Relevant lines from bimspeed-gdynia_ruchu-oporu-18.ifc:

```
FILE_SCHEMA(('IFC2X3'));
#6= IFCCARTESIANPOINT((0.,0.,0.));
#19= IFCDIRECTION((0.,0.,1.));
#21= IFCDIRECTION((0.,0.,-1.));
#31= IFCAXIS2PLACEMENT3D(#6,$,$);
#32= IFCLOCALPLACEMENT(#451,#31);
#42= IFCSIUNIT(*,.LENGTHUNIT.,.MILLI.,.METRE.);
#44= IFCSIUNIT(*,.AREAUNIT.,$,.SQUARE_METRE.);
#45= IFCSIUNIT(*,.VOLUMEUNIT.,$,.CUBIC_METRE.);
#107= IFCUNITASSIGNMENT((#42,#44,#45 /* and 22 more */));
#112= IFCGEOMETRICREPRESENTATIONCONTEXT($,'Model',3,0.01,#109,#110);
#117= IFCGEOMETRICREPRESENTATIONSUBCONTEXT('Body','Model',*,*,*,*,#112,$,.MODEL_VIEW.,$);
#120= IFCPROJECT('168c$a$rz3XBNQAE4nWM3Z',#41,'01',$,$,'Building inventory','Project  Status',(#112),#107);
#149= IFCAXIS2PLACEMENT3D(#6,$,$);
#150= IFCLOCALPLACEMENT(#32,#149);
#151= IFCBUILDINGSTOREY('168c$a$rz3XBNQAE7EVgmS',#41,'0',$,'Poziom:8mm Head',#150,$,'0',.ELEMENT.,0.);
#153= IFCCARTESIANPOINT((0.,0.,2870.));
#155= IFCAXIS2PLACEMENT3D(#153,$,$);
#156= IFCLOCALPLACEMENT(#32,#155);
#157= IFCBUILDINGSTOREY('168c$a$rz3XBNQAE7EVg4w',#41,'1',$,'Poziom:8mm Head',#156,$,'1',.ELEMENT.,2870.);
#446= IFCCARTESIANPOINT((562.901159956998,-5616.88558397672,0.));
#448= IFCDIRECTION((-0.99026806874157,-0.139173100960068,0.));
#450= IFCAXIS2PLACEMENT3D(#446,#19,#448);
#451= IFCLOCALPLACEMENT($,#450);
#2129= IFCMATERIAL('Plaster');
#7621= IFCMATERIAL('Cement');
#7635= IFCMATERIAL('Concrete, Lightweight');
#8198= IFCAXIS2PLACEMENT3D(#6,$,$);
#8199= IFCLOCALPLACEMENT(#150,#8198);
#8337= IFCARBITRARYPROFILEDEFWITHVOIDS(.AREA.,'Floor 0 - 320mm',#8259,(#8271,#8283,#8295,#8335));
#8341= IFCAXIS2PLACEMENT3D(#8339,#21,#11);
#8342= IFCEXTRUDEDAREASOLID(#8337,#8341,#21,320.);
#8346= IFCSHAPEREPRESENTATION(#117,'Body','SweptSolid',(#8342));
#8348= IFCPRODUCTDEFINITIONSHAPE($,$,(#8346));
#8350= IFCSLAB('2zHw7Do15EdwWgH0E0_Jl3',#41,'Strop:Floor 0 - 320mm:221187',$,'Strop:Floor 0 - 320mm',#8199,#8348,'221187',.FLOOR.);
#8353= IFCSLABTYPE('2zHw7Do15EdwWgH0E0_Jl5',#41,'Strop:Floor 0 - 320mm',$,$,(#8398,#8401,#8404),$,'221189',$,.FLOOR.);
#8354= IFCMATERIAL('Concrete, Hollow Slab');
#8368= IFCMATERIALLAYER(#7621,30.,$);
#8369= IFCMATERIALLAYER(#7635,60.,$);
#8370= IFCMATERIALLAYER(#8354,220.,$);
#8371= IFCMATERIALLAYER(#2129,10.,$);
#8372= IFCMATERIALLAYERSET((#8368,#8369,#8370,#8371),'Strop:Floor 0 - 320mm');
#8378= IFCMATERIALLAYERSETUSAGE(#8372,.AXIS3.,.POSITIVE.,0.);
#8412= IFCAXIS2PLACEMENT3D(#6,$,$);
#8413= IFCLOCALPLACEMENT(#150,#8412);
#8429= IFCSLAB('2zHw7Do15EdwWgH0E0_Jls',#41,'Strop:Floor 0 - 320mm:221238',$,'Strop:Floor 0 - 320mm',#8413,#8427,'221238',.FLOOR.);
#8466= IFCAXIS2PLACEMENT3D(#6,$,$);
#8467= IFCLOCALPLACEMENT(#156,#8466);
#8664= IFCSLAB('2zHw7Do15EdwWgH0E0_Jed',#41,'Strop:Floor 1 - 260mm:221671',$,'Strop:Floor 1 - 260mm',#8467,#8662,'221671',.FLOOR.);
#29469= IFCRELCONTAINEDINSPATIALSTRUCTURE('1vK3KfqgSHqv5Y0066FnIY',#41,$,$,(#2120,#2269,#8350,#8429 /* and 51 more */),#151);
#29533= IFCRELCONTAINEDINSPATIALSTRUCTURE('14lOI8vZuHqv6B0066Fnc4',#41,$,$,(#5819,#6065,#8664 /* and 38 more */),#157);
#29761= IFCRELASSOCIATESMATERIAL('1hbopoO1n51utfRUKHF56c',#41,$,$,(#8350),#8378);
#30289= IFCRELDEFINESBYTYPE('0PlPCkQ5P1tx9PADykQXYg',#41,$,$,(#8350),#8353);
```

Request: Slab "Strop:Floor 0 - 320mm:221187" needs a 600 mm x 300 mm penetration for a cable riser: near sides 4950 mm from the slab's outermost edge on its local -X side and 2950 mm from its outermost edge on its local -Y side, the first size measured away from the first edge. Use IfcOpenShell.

```python
import numpy as np
import ifcopenshell
import ifcopenshell.api.feature
import ifcopenshell.api.geometry
import ifcopenshell.api.root
import ifcopenshell.geom
import ifcopenshell.util.placement
import ifcopenshell.util.representation
import ifcopenshell.util.shape
import ifcopenshell.util.unit

model = ifcopenshell.open("bimspeed-gdynia_ruchu-oporu-18.ifc")
unit_scale = ifcopenshell.util.unit.calculate_unit_scale(model)
settings = ifcopenshell.geom.settings()


def volume(element):
    """Net volume in cubic metres, openings subtracted."""
    shape = ifcopenshell.geom.create_shape(settings, element)
    return ifcopenshell.util.shape.get_volume(shape.geometry)


slab = model.by_guid("2zHw7Do15EdwWgH0E0_Jl3")
before = volume(slab)

# Extent in the slab's own axes, in metres. The edges named are its -X and -Y sides.
slab_shape = ifcopenshell.geom.create_shape(settings, slab)
vertices = ifcopenshell.util.shape.get_vertices(slab_shape.geometry)
x_min, y_min, bottom = vertices.min(axis=0)
top = vertices[:, 2].max()

opening = ifcopenshell.api.root.create_entity(model, ifc_class="IfcOpeningElement", name="Cable riser opening")
context = ifcopenshell.util.representation.get_context(model, "Model", "Body", "MODEL_VIEW")
width, depth = 0.6, 0.3
outline = [(0.0, 0.0), (width, 0.0), (width, depth), (0.0, depth), (0.0, 0.0)]
# Overshoot both faces by 50 mm so the cut is clean.
shape = ifcopenshell.api.geometry.add_slab_representation(
    model, context=context, depth=top - bottom + 0.1, polyline=outline
)
ifcopenshell.api.geometry.assign_representation(model, product=opening, representation=shape)

matrix = ifcopenshell.util.placement.get_local_placement(slab.ObjectPlacement)
matrix[:, 3] = matrix @ np.append(np.array([x_min + 4.95, y_min + 2.95, bottom - 0.05]) / unit_scale, 1.0)
ifcopenshell.api.geometry.edit_object_placement(model, product=opening, matrix=matrix, is_si=False)
ifcopenshell.api.feature.add_feature(model, feature=opening, element=slab)

after = volume(slab)

print(f"slab volume {before:.3f} -> {after:.3f} m3")

model.write("bimspeed-gdynia_ruchu-oporu-18-out.ifc")
```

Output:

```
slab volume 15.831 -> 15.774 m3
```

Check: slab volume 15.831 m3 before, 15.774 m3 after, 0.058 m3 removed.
